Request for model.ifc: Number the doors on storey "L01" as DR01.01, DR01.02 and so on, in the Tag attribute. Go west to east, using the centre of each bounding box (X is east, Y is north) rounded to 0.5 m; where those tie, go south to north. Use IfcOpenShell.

First a look at what the model holds.

```python
import ifcopenshell
import ifcopenshell.util.element
import ifcopenshell.util.placement

model = ifcopenshell.open("model.ifc")
print(model.schema)
storey = next(s for s in model.by_type("IfcBuildingStorey") if s.Name == "L01")
doors = [e for e in ifcopenshell.util.element.get_decomposition(storey) if e.is_a("IfcDoor")]
for e in sorted(doors, key=lambda e: e.id()):
    origin = ifcopenshell.util.placement.get_local_placement(e.ObjectPlacement)[:3, 3]
    print(e.id(), e.Tag, e.Name, origin.round(2) + 0.0, sep=" | ")
```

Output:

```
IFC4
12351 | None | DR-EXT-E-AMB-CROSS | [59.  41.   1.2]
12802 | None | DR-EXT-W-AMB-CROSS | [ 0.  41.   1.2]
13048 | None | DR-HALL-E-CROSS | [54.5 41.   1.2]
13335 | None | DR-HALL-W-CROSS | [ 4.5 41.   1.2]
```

```python
import ifcopenshell
import ifcopenshell.geom
import ifcopenshell.util.element
import ifcopenshell.util.shape

model = ifcopenshell.open("model.ifc")
settings = ifcopenshell.geom.settings()
settings.set("use-world-coords", True)


def centre(element):
    shape = ifcopenshell.geom.create_shape(settings, element)
    return ifcopenshell.util.shape.get_bbox_centroid(shape.geometry)


storey = next(s for s in model.by_type("IfcBuildingStorey") if s.Name == "L01")
doors = [e for e in ifcopenshell.util.element.get_decomposition(storey) if e.is_a("IfcDoor")]

# Insertion points can sit at a corner or the storey origin, so sort by the geometry (in metres).
centres = {e: centre(e) for e in doors}
doors.sort(key=lambda e: (round(centres[e][0] / 0.5), centres[e][1]))

for i, e in enumerate(doors, start=1):
    number = f"DR01.{i:02d}"
    e.Tag = number
    print(e.id(), number)

model.write("model_rev.ifc")
```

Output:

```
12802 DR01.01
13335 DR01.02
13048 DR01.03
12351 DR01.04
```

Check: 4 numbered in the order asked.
